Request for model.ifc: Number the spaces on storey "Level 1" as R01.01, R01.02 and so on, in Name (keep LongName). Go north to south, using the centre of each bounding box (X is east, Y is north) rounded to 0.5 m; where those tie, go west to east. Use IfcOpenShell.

First a look at what the model holds.

```python
import ifcopenshell
import ifcopenshell.util.element
import ifcopenshell.util.placement

model = ifcopenshell.open("model.ifc")
print(model.schema)
storey = next(s for s in model.by_type("IfcBuildingStorey") if s.Name == "Level 1")
spaces = [e for e in ifcopenshell.util.element.get_decomposition(storey) if e.is_a("IfcSpace")]
for e in sorted(spaces, key=lambda e: e.id()):
    origin = ifcopenshell.util.placement.get_local_placement(e.ObjectPlacement)[:3, 3]
    print(e.id(), e.Name, e.LongName, origin.round(2) + 0.0, sep=" | ")
```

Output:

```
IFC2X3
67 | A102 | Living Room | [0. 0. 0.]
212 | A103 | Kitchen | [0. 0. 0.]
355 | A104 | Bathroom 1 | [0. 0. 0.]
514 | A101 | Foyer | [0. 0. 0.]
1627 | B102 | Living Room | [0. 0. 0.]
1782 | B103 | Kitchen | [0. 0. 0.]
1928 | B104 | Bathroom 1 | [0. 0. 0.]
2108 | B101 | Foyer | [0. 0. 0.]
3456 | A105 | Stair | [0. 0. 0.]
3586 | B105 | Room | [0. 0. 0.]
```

```python
import ifcopenshell
import ifcopenshell.geom
import ifcopenshell.util.element
import ifcopenshell.util.shape

model = ifcopenshell.open("model.ifc")
settings = ifcopenshell.geom.settings()
settings.set("use-world-coords", True)


def centre(element):
    shape = ifcopenshell.geom.create_shape(settings, element)
    return ifcopenshell.util.shape.get_bbox_centroid(shape.geometry)


storey = next(s for s in model.by_type("IfcBuildingStorey") if s.Name == "Level 1")
spaces = [e for e in ifcopenshell.util.element.get_decomposition(storey) if e.is_a("IfcSpace")]

# Insertion points can sit at a corner or the storey origin, so sort by the geometry (in metres).
centres = {e: centre(e) for e in spaces}
spaces.sort(key=lambda e: (-round(centres[e][1] / 0.5), centres[e][0]))

for i, e in enumerate(spaces, start=1):
    number = f"R01.{i:02d}"
    e.Name = number
    print(e.id(), number)

model.write("model_v2.ifc")
```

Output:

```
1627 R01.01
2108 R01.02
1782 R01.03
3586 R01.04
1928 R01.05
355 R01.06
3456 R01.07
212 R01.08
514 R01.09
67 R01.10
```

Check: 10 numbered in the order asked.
